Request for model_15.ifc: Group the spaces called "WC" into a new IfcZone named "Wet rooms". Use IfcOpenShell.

First a look at what the model holds.

```python
import ifcopenshell

model = ifcopenshell.open("model_15.ifc")
print(model.schema)
seen = {}
for space in model.by_type("IfcSpace"):
    seen[space.LongName] = seen.get(space.LongName, 0) + 1
for name, count in sorted(seen.items(), key=str):
    print(count, "x", name)
print("zones:", [z.Name for z in model.by_type("IfcZone")][:20])
```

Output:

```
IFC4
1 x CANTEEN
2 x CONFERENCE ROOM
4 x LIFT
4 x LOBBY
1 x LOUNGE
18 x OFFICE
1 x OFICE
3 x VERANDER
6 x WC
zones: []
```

```python
import ifcopenshell
import ifcopenshell.api.group
import ifcopenshell.api.root

model = ifcopenshell.open("model_15.ifc")

names = {"WC"}
spaces = [s for s in model.by_type("IfcSpace") if s.LongName in names]

zone = ifcopenshell.api.root.create_entity(model, ifc_class="IfcZone", name="Wet rooms")
ifcopenshell.api.group.assign_group(model, products=spaces, group=zone)
print(len(spaces), "spaces in", zone.Name)

model.write("model_15_v2.ifc")
```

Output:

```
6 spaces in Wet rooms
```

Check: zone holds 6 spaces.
